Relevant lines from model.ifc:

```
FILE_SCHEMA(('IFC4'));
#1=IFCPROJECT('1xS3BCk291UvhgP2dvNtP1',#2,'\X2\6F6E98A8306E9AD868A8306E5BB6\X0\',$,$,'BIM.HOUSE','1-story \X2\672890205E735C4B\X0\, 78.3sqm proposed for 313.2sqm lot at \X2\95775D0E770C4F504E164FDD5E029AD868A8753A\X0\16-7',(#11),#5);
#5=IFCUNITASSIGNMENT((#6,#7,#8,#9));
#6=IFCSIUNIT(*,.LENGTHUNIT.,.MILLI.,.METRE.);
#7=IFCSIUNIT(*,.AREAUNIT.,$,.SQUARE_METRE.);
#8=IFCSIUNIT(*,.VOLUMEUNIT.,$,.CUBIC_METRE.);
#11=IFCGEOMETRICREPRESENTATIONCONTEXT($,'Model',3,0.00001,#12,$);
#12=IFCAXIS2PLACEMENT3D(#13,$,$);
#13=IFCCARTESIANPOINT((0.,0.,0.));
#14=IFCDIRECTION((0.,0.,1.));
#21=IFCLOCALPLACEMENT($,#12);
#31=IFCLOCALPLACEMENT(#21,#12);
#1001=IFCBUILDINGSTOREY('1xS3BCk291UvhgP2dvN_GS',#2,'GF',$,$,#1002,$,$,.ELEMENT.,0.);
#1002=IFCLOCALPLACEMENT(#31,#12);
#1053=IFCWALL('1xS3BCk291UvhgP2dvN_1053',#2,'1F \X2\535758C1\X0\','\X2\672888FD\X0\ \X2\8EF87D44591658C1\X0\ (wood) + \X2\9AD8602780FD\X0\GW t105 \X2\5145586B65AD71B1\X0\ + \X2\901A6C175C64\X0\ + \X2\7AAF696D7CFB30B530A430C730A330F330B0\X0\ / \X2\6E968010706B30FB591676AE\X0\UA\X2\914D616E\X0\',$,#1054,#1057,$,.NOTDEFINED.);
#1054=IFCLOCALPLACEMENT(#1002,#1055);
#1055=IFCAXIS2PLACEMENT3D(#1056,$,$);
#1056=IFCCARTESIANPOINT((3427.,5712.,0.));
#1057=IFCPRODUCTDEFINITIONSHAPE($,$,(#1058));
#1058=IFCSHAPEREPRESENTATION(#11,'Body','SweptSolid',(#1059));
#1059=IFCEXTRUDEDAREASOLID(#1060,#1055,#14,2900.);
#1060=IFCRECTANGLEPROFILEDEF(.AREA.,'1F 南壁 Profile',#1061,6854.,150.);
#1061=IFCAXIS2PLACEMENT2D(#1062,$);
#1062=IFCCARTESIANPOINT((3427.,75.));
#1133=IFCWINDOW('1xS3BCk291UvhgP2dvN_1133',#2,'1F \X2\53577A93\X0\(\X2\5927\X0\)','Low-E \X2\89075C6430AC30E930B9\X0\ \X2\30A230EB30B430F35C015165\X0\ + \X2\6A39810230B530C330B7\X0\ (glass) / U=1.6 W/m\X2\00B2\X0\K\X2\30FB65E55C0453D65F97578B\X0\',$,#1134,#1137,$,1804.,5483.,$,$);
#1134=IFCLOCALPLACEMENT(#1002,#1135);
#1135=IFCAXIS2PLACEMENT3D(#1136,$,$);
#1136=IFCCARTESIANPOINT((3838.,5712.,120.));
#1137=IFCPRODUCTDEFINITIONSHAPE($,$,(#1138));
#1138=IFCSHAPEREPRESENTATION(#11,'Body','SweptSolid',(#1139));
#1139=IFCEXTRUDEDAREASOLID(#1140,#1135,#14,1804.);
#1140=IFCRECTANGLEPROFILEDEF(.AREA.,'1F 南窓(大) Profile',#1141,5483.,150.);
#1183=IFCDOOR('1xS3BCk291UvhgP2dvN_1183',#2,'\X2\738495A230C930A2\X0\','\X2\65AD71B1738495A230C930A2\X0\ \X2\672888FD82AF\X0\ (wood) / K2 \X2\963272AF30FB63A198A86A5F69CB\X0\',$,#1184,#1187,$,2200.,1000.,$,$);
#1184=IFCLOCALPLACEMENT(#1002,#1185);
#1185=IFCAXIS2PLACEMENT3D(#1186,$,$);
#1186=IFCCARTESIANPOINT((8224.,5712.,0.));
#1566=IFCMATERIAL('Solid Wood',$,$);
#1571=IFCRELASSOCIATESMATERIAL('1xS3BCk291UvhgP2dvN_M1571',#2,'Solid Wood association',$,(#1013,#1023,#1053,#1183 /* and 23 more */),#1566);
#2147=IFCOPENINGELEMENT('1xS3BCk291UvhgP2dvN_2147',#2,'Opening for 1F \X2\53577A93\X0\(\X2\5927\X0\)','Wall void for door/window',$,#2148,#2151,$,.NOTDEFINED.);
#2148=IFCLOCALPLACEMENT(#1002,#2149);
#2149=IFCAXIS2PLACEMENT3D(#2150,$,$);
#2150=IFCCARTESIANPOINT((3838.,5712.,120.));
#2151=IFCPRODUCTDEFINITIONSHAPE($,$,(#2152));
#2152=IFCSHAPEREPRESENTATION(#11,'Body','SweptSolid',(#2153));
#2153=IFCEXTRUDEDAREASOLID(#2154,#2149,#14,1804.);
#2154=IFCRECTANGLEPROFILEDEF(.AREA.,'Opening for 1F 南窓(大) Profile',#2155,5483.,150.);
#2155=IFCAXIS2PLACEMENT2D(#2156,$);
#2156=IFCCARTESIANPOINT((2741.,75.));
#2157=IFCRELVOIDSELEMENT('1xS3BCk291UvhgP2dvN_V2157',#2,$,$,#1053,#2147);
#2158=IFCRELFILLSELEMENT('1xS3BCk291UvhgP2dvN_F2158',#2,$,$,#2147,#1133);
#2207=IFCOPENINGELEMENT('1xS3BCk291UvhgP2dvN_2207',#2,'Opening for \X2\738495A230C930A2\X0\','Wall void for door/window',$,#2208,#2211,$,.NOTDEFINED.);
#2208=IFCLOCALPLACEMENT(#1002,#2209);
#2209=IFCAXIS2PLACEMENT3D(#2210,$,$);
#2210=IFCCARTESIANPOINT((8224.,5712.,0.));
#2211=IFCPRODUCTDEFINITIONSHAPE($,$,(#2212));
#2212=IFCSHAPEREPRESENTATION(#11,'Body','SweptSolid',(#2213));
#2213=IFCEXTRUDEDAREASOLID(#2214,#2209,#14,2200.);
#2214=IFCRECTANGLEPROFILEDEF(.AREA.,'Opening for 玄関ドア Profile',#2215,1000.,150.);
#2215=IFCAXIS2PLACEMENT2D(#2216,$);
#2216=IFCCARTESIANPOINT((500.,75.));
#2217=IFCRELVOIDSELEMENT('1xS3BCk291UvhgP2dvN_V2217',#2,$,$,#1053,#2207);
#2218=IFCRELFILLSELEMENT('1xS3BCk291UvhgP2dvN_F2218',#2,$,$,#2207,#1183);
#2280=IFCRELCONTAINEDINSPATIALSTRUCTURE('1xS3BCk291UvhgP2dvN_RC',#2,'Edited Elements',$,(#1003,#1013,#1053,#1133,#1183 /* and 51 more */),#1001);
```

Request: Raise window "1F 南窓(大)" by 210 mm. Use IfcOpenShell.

```python
import numpy as np
import ifcopenshell
import ifcopenshell.api.geometry
import ifcopenshell.util.placement
import ifcopenshell.util.unit

model = ifcopenshell.open("model.ifc")
unit_scale = ifcopenshell.util.unit.calculate_unit_scale(model)

window = model.by_guid("1xS3BCk291UvhgP2dvN_1133")
opening = window.FillsVoids[0].RelatingOpeningElement
dz = 0.21 / unit_scale

shift = np.array([0.0, 0.0, dz])
# The window is not placed relative to its opening, so move both.
for product in (opening, window):
    matrix = ifcopenshell.util.placement.get_local_placement(product.ObjectPlacement)
    matrix[:3, 3] += shift
    ifcopenshell.api.geometry.edit_object_placement(model, product=product, matrix=matrix, is_si=False)

print(f"moved by {dz * unit_scale:+.3f} m")

model.write("model_edited.ifc")
```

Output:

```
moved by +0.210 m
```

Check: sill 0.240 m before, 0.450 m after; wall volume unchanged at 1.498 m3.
